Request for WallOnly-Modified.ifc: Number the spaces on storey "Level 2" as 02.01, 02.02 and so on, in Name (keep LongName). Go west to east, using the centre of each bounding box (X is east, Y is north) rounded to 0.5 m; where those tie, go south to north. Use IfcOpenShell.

First a look at what the model holds.

```python
import ifcopenshell
import ifcopenshell.util.element
import ifcopenshell.util.placement

model = ifcopenshell.open("WallOnly-Modified.ifc")
print(model.schema)
storey = next(s for s in model.by_type("IfcBuildingStorey") if s.Name == "Level 2")
spaces = [e for e in ifcopenshell.util.element.get_decomposition(storey) if e.is_a("IfcSpace")]
for e in sorted(spaces, key=lambda e: e.id()):
    origin = ifcopenshell.util.placement.get_local_placement(e.ObjectPlacement)[:3, 3]
    print(e.id(), e.Name, e.LongName, origin.round(2) + 0.0, sep=" | ")
```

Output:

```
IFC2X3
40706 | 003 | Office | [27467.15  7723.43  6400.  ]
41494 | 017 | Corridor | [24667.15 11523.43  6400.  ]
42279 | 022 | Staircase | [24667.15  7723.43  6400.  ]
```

```python
import ifcopenshell
import ifcopenshell.geom
import ifcopenshell.util.element
import ifcopenshell.util.shape

model = ifcopenshell.open("WallOnly-Modified.ifc")
settings = ifcopenshell.geom.settings()
settings.set("use-world-coords", True)


def centre(element):
    shape = ifcopenshell.geom.create_shape(settings, element)
    return ifcopenshell.util.shape.get_bbox_centroid(shape.geometry)


storey = next(s for s in model.by_type("IfcBuildingStorey") if s.Name == "Level 2")
spaces = [e for e in ifcopenshell.util.element.get_decomposition(storey) if e.is_a("IfcSpace")]

# Insertion points can sit at a corner or the storey origin, so sort by the geometry (in metres).
centres = {e: centre(e) for e in spaces}
spaces.sort(key=lambda e: (round(centres[e][0] / 0.5), centres[e][1]))

for i, e in enumerate(spaces, start=1):
    number = f"02.{i:02d}"
    e.Name = number
    print(e.id(), number)

model.write("WallOnly-Modified_v2.ifc")
```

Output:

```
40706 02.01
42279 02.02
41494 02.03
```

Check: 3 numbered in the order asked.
